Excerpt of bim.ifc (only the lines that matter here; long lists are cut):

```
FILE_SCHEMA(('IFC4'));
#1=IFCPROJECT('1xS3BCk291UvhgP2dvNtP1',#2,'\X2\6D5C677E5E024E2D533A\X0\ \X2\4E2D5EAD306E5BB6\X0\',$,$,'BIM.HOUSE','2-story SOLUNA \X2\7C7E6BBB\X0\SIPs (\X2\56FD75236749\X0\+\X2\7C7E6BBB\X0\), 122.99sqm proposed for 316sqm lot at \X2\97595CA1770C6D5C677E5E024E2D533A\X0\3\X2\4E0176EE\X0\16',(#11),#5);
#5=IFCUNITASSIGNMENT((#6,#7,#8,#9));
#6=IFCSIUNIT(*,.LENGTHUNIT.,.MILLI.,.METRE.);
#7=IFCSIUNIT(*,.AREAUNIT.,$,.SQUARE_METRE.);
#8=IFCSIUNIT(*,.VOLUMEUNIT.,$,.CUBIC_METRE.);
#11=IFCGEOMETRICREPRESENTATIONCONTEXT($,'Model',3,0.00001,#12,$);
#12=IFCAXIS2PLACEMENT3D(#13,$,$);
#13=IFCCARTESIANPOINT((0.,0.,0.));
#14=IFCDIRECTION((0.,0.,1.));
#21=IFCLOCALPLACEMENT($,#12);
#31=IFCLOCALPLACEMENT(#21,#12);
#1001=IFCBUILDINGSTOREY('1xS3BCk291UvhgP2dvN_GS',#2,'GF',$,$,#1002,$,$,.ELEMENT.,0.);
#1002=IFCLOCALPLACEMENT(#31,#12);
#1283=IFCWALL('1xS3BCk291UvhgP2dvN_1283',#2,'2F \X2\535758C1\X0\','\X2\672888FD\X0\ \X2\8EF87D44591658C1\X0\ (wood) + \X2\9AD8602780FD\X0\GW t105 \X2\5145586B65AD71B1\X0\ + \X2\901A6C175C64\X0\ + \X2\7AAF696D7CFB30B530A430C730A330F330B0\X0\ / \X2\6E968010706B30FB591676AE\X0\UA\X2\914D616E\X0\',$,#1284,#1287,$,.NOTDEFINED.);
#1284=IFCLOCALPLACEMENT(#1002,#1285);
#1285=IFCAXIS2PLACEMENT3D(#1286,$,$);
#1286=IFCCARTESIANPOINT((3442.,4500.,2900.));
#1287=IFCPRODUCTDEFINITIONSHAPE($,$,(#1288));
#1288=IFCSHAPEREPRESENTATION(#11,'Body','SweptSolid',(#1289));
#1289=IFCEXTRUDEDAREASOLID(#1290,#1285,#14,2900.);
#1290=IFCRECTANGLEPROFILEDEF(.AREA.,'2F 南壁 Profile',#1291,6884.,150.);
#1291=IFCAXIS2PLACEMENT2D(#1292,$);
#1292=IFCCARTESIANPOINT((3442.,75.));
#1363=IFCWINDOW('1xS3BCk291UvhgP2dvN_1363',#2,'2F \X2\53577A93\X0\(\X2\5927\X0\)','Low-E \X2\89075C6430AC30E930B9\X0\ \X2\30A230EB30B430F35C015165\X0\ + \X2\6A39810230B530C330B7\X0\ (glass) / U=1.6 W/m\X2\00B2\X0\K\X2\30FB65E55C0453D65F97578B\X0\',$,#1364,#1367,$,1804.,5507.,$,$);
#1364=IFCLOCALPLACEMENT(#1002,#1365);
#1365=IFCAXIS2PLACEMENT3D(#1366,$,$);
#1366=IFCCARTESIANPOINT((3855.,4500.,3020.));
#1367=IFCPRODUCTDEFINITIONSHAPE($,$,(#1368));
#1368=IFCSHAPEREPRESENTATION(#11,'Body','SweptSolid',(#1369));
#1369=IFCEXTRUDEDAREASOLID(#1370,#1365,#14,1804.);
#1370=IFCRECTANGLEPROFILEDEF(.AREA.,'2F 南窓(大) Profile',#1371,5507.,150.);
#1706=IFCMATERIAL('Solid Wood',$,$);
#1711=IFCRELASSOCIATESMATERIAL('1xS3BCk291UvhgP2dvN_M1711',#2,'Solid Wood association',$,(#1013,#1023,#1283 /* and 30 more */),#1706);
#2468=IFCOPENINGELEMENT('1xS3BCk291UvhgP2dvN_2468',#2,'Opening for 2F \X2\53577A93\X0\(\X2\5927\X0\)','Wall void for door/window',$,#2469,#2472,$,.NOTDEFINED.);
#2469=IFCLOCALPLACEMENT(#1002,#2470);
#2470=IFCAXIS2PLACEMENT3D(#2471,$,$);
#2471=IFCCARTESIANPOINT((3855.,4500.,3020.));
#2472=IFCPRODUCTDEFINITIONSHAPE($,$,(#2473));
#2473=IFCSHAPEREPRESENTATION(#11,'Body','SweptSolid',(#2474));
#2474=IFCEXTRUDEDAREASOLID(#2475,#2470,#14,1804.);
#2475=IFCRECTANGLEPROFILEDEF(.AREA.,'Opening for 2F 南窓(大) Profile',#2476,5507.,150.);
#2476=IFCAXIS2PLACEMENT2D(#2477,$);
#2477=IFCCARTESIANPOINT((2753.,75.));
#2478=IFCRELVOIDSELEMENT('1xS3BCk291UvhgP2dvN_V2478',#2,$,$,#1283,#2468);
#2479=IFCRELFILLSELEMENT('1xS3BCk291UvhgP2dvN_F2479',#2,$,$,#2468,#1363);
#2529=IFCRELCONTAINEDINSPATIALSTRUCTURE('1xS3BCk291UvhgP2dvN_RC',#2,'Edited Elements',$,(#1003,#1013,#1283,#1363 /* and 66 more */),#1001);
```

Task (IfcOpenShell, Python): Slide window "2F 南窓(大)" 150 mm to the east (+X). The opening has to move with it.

```python
import ifcopenshell
import ifcopenshell.api.geometry
import ifcopenshell.util.placement
import ifcopenshell.util.unit

model = ifcopenshell.open("bim.ifc")
unit_scale = ifcopenshell.util.unit.calculate_unit_scale(model)

window = model.by_guid("1xS3BCk291UvhgP2dvN_1363")
opening = window.FillsVoids[0].RelatingOpeningElement
wall = opening.VoidsElements[0].RelatingBuildingElement

wall_matrix = ifcopenshell.util.placement.get_local_placement(wall.ObjectPlacement)
shift = wall_matrix[:3, 0] * 0.15 / unit_scale
before = ifcopenshell.util.placement.get_local_placement(window.ObjectPlacement)[:3, 3].copy()

# The window is not placed relative to its opening, so move both.
for product in (opening, window):
    matrix = ifcopenshell.util.placement.get_local_placement(product.ObjectPlacement)
    matrix[:3, 3] += shift
    ifcopenshell.api.geometry.edit_object_placement(model, product=product, matrix=matrix, is_si=False)

after = ifcopenshell.util.placement.get_local_placement(window.ObjectPlacement)[:3, 3]
print("window moved by", (after - before).round(3) + 0.0)

model.write("bim_rev.ifc")
```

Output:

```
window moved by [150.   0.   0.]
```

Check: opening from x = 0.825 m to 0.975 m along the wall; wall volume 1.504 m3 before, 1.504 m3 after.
